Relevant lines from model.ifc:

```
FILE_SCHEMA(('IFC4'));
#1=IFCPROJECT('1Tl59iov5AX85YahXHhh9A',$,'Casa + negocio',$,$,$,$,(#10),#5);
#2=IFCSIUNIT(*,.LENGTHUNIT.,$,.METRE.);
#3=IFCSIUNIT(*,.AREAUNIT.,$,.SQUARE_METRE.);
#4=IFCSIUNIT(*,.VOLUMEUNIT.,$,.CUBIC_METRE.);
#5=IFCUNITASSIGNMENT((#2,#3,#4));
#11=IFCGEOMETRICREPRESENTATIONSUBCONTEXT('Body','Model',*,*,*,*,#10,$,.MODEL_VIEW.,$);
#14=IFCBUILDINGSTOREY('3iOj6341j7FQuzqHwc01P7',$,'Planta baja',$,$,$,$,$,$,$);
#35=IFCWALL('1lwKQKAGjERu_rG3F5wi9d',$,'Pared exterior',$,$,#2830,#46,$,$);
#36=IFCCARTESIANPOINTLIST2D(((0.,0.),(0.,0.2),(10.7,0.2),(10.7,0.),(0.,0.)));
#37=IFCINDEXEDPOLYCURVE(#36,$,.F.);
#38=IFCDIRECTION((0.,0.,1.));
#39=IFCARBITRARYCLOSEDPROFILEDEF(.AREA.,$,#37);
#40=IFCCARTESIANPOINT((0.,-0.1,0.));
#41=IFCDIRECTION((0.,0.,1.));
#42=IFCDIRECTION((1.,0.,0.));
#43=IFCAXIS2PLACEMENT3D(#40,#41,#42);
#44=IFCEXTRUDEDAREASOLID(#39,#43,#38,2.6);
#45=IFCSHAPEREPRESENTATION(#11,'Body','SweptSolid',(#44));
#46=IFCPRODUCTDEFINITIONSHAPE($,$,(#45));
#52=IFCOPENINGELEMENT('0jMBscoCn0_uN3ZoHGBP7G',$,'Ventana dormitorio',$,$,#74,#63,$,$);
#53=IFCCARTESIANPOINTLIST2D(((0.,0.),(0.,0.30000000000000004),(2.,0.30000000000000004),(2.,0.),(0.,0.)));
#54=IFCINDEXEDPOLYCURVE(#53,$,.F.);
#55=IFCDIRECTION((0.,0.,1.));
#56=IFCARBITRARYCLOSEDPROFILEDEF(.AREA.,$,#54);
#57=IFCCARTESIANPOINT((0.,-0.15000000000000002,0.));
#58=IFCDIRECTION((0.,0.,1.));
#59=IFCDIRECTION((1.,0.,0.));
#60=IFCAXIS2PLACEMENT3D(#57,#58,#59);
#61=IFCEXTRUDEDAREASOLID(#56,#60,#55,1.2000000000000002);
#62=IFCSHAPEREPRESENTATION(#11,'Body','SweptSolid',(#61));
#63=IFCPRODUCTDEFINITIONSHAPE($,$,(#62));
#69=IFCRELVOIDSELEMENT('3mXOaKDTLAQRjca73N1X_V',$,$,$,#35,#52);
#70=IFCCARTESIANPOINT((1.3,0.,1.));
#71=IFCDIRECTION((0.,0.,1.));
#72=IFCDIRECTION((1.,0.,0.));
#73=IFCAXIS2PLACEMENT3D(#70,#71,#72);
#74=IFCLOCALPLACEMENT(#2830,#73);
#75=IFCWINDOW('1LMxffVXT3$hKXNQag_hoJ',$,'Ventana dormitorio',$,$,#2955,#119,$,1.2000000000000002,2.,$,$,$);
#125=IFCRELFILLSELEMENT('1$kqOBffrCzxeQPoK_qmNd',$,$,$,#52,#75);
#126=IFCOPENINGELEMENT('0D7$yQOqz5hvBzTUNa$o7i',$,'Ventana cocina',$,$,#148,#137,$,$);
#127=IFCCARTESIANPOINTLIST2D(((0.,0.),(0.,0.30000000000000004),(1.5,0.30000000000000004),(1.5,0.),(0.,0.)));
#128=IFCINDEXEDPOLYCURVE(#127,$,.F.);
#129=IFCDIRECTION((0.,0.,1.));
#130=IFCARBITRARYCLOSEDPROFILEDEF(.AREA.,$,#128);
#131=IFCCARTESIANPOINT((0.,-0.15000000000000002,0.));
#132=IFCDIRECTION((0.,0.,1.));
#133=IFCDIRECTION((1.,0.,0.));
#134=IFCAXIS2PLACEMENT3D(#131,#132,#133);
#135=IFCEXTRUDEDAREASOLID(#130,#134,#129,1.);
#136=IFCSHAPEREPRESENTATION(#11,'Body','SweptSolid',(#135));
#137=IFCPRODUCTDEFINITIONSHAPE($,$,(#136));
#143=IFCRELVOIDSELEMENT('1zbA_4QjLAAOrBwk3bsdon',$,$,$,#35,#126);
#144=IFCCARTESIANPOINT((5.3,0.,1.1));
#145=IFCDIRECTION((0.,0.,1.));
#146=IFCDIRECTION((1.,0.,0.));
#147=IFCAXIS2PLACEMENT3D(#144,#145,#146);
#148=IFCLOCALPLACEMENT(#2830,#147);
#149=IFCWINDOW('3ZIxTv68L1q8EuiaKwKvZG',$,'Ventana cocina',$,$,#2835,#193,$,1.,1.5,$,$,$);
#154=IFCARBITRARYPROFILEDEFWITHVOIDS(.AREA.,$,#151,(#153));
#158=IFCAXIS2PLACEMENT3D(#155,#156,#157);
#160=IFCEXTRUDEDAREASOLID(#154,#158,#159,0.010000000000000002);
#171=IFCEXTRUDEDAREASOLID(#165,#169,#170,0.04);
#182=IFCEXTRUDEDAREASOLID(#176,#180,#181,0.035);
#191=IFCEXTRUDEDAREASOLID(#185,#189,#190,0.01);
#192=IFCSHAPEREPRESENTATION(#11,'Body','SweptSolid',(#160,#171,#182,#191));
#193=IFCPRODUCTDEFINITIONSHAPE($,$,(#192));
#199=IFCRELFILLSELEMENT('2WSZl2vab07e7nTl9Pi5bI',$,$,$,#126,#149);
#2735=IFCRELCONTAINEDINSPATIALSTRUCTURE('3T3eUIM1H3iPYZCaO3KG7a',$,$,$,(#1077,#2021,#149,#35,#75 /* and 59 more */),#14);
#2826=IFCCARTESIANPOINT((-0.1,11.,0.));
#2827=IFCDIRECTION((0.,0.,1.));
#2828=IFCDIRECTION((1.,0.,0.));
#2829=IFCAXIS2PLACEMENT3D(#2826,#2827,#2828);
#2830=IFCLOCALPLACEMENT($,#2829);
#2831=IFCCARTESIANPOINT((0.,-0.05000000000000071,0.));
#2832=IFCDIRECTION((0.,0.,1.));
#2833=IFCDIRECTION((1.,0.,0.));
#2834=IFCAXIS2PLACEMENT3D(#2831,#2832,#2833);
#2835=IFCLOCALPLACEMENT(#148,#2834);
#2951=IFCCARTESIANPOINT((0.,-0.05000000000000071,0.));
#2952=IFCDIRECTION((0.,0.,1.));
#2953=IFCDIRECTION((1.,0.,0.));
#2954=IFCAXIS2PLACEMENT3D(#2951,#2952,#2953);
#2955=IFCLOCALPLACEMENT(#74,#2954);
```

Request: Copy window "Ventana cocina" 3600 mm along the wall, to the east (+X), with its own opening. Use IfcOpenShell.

```python
import ifcopenshell
import ifcopenshell.api.feature
import ifcopenshell.api.geometry
import ifcopenshell.api.root
import ifcopenshell.geom
import ifcopenshell.util.element
import ifcopenshell.util.placement
import ifcopenshell.util.shape
import ifcopenshell.util.unit

model = ifcopenshell.open("model.ifc")
unit_scale = ifcopenshell.util.unit.calculate_unit_scale(model)
settings = ifcopenshell.geom.settings()


def volume(element):
    """Net volume in cubic metres, openings subtracted."""
    shape = ifcopenshell.geom.create_shape(settings, element)
    return ifcopenshell.util.shape.get_volume(shape.geometry)


window = model.by_guid("3ZIxTv68L1q8EuiaKwKvZG")
opening = window.FillsVoids[0].RelatingOpeningElement
wall = opening.VoidsElements[0].RelatingBuildingElement
before = volume(wall)
shift = ifcopenshell.util.placement.get_local_placement(wall.ObjectPlacement)[:3, 0] * 3.6 / unit_scale

# copy_class copies the void relationship, type, container and properties, but no geometry.
new_opening = ifcopenshell.api.root.copy_class(model, product=opening)
new_opening.Representation = ifcopenshell.util.element.copy_deep(
    model, opening.Representation, exclude=["IfcGeometricRepresentationContext", "IfcRepresentationMap"]
)
new_window = ifcopenshell.api.root.copy_class(model, product=window)
new_window.Representation = ifcopenshell.util.element.copy_deep(
    model, window.Representation, exclude=["IfcGeometricRepresentationContext", "IfcRepresentationMap"]
)
ifcopenshell.api.feature.add_filling(model, opening=new_opening, element=new_window)

for old, new in ((opening, new_opening), (window, new_window)):
    matrix = ifcopenshell.util.placement.get_local_placement(old.ObjectPlacement)
    matrix[:3, 3] += shift
    ifcopenshell.api.geometry.edit_object_placement(model, product=new, matrix=matrix, is_si=False)

after = volume(wall)

print(f"wall volume {before:.3f} -> {after:.3f} m3")

model.write("model_edited.ifc")
```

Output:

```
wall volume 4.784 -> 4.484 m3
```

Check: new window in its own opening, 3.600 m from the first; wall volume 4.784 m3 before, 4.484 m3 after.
